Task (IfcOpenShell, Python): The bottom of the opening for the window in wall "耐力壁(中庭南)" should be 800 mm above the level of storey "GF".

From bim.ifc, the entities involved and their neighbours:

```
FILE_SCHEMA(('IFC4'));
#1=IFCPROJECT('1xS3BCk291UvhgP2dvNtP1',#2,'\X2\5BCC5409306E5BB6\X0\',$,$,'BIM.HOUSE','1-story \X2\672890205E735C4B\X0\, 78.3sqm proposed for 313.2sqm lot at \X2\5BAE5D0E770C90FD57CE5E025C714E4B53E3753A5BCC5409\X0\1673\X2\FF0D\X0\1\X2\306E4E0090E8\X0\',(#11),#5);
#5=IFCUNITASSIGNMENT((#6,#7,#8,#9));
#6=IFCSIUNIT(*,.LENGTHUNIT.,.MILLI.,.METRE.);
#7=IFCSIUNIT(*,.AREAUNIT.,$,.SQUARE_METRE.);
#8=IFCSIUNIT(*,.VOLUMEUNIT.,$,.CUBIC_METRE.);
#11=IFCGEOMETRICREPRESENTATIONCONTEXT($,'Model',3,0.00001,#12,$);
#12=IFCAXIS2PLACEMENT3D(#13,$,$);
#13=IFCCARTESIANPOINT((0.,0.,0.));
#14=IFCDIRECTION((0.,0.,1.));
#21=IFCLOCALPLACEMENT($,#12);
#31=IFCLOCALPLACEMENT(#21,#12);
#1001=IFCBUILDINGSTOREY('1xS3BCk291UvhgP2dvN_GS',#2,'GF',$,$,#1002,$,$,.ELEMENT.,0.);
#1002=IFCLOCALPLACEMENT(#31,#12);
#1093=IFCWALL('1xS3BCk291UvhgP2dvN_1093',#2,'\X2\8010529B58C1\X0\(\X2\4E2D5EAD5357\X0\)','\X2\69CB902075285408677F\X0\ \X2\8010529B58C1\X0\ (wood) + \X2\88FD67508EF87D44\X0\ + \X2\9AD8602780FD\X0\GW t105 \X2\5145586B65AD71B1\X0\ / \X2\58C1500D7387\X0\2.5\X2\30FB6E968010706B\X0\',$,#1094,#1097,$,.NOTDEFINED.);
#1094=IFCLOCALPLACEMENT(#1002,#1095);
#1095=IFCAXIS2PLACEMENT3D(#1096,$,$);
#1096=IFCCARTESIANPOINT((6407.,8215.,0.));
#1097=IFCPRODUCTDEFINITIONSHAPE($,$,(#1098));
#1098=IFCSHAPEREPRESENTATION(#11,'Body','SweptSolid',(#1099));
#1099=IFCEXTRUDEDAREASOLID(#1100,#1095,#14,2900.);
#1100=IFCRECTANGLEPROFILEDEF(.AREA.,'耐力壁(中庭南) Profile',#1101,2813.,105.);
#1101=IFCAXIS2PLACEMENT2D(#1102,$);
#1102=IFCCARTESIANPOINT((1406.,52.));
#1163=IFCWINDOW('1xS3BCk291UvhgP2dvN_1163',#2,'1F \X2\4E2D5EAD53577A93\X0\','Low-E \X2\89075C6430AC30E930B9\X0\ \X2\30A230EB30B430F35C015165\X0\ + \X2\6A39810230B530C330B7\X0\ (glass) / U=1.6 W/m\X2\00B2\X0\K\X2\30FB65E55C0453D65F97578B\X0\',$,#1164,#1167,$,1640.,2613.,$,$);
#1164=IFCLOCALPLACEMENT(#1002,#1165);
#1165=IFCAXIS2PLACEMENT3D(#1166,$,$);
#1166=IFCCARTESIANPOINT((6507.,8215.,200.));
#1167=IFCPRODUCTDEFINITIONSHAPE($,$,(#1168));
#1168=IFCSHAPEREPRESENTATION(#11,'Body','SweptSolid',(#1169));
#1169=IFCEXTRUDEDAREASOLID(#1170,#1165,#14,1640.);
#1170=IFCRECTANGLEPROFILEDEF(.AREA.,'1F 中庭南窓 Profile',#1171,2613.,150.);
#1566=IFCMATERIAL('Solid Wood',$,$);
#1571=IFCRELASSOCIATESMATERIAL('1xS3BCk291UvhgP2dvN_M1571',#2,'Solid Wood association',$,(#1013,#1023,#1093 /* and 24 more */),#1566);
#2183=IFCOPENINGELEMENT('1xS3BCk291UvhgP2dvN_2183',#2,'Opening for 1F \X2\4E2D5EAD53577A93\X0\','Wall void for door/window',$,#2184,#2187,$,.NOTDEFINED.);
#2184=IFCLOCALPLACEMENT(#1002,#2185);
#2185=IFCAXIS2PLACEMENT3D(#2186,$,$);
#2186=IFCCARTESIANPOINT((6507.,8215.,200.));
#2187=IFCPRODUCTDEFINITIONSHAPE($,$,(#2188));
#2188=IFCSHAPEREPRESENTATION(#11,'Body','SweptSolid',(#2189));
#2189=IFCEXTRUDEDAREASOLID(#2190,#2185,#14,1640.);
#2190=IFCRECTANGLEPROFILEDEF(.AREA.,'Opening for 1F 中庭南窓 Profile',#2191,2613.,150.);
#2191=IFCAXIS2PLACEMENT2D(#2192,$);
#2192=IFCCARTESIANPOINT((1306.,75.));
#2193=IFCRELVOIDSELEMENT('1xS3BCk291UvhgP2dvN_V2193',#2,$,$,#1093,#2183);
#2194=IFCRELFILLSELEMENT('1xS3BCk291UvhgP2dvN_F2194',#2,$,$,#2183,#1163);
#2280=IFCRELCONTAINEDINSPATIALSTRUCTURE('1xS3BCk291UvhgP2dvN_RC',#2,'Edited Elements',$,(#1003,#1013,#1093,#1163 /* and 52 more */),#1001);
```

```python
import numpy as np
import ifcopenshell
import ifcopenshell.api.geometry
import ifcopenshell.geom
import ifcopenshell.util.element
import ifcopenshell.util.placement
import ifcopenshell.util.shape
import ifcopenshell.util.unit

model = ifcopenshell.open("bim.ifc")
unit_scale = ifcopenshell.util.unit.calculate_unit_scale(model)

window = model.by_id(1163)
opening = window.FillsVoids[0].RelatingOpeningElement
storey = ifcopenshell.util.element.get_container(window, ifc_class="IfcBuildingStorey")
level = ifcopenshell.util.placement.get_local_placement(storey.ObjectPlacement)[2, 3]

# The opening's origin need not be at the sill, so measure its lowest point.
shape = ifcopenshell.geom.create_shape(ifcopenshell.geom.settings(), opening)
bottom = ifcopenshell.util.shape.get_shape_bottom_elevation(shape, shape.geometry) / unit_scale
dz = level + 800.0 - bottom

shift = np.array([0.0, 0.0, dz])
# The window is not placed relative to its opening, so move both.
for product in (opening, window):
    matrix = ifcopenshell.util.placement.get_local_placement(product.ObjectPlacement)
    matrix[:3, 3] += shift
    ifcopenshell.api.geometry.edit_object_placement(model, product=product, matrix=matrix, is_si=False)

print(f"moved by {dz * unit_scale:+.3f} m")

model.write("bim_v2.ifc")
```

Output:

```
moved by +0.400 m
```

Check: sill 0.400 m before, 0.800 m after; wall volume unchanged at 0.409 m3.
